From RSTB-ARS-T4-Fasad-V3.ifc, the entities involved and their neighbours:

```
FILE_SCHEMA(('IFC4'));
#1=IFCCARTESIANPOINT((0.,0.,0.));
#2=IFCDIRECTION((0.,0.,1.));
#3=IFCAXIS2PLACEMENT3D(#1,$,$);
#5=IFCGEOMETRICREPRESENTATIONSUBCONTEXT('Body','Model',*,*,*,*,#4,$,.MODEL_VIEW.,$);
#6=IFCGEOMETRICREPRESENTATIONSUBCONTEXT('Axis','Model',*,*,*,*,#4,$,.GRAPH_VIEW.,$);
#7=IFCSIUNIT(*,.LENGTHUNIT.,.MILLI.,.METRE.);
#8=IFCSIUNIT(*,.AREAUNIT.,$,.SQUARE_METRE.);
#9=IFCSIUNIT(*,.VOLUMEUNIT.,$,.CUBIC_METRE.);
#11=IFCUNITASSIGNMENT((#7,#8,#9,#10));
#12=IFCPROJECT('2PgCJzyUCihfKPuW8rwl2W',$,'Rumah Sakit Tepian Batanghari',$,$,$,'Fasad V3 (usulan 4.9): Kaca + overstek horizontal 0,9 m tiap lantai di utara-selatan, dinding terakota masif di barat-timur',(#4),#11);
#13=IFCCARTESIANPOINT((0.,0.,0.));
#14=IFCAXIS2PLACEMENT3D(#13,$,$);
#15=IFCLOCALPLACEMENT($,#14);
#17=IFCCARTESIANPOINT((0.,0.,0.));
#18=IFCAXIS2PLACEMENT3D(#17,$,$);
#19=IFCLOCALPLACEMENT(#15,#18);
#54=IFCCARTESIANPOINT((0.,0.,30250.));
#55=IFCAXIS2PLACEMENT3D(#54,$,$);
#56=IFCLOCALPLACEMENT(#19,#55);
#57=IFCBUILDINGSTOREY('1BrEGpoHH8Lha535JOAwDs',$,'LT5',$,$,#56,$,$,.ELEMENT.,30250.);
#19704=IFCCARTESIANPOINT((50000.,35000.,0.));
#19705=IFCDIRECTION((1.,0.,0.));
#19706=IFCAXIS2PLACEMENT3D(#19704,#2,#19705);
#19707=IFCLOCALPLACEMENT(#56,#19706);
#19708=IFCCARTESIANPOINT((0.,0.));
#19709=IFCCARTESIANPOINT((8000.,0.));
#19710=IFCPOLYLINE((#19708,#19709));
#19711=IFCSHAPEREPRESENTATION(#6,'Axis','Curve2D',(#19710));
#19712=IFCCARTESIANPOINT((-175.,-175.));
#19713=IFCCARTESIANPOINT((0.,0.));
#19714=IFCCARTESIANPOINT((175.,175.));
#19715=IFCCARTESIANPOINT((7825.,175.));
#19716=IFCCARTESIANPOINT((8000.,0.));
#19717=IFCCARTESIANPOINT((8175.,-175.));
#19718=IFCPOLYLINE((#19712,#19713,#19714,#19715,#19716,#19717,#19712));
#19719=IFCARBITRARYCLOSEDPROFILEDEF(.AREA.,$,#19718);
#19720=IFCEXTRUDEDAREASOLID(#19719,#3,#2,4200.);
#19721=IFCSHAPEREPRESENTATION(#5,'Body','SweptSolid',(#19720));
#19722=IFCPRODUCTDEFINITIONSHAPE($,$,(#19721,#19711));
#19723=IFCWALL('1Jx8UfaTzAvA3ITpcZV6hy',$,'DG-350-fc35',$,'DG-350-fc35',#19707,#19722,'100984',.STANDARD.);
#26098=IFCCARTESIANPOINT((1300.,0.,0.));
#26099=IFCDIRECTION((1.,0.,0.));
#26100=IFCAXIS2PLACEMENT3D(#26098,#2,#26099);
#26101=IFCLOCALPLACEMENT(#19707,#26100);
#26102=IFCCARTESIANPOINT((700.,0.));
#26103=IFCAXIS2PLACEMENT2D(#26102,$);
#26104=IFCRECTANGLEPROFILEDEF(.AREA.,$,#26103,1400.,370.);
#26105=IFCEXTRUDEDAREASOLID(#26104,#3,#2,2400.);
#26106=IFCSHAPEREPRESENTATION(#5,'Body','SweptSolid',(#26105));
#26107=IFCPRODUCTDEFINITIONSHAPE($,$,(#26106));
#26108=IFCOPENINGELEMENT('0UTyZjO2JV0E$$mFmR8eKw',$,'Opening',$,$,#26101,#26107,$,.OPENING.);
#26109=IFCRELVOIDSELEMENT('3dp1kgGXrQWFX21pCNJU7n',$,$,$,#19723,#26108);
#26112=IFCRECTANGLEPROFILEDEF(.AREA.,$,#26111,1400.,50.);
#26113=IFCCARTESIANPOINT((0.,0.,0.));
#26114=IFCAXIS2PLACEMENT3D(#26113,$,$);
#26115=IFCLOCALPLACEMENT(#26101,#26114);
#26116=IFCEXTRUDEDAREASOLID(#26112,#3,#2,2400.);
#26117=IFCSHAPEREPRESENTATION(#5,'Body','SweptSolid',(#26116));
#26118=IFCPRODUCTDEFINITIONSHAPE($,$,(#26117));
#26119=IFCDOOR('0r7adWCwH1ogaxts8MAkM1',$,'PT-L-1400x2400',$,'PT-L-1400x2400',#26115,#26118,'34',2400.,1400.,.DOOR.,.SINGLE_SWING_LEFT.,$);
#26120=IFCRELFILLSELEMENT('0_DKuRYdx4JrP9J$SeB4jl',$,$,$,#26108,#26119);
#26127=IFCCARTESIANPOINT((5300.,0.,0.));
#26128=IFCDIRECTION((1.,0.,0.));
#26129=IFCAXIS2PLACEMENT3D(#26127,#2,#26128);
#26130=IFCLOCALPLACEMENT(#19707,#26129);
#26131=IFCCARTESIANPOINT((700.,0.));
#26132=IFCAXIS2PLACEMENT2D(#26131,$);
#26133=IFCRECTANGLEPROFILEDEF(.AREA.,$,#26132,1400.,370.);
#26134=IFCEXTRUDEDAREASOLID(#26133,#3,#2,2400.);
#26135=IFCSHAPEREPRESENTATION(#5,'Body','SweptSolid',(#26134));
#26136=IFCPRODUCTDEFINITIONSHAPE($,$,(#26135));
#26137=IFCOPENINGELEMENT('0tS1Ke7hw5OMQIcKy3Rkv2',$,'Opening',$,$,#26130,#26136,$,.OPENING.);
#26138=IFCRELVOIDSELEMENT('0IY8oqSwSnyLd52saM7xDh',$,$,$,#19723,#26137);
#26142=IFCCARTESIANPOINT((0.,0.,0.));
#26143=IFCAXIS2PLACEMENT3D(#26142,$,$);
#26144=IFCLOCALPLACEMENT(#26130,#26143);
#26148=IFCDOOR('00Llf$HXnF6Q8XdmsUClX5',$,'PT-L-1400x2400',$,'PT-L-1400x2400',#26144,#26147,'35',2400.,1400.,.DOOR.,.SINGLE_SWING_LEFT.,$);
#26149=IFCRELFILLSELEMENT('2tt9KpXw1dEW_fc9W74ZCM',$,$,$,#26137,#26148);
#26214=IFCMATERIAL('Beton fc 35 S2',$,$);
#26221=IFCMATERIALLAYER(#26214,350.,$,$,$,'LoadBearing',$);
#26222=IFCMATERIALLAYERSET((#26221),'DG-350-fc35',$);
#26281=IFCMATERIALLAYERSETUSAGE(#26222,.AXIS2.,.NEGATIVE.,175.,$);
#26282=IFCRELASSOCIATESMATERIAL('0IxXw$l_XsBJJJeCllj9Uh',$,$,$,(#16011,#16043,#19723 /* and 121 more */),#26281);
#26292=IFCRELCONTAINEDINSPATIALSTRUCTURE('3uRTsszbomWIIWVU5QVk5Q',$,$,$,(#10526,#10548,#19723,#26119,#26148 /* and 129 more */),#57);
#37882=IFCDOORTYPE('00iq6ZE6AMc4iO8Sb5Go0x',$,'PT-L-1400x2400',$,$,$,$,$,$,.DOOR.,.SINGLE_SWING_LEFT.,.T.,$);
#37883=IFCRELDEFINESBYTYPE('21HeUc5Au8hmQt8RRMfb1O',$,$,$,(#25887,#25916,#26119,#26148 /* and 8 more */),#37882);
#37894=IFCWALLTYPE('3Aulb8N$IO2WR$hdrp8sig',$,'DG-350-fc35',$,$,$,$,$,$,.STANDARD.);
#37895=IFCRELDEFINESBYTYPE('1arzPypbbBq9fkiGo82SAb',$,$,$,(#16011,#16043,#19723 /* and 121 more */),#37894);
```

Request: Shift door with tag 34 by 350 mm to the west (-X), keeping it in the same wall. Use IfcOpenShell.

```python
import ifcopenshell
import ifcopenshell.api.geometry
import ifcopenshell.util.placement
import ifcopenshell.util.unit

model = ifcopenshell.open("RSTB-ARS-T4-Fasad-V3.ifc")
unit_scale = ifcopenshell.util.unit.calculate_unit_scale(model)

door = model.by_guid("0r7adWCwH1ogaxts8MAkM1")
opening = door.FillsVoids[0].RelatingOpeningElement
wall = opening.VoidsElements[0].RelatingBuildingElement

wall_matrix = ifcopenshell.util.placement.get_local_placement(wall.ObjectPlacement)
shift = wall_matrix[:3, 0] * -0.35 / unit_scale
before = ifcopenshell.util.placement.get_local_placement(door.ObjectPlacement)[:3, 3].copy()

# The door is placed relative to its opening, so it follows when the opening moves.
matrix = ifcopenshell.util.placement.get_local_placement(opening.ObjectPlacement)
matrix[:3, 3] += shift
ifcopenshell.api.geometry.edit_object_placement(
    model, product=opening, matrix=matrix, is_si=False, should_transform_children=True
)

after = ifcopenshell.util.placement.get_local_placement(door.ObjectPlacement)[:3, 3]
print("door moved by", (after - before).round(3) + 0.0)

model.write("RSTB-ARS-T4-Fasad-V3_v2.ifc")
```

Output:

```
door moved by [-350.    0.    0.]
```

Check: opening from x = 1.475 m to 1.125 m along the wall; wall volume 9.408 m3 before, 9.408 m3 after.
